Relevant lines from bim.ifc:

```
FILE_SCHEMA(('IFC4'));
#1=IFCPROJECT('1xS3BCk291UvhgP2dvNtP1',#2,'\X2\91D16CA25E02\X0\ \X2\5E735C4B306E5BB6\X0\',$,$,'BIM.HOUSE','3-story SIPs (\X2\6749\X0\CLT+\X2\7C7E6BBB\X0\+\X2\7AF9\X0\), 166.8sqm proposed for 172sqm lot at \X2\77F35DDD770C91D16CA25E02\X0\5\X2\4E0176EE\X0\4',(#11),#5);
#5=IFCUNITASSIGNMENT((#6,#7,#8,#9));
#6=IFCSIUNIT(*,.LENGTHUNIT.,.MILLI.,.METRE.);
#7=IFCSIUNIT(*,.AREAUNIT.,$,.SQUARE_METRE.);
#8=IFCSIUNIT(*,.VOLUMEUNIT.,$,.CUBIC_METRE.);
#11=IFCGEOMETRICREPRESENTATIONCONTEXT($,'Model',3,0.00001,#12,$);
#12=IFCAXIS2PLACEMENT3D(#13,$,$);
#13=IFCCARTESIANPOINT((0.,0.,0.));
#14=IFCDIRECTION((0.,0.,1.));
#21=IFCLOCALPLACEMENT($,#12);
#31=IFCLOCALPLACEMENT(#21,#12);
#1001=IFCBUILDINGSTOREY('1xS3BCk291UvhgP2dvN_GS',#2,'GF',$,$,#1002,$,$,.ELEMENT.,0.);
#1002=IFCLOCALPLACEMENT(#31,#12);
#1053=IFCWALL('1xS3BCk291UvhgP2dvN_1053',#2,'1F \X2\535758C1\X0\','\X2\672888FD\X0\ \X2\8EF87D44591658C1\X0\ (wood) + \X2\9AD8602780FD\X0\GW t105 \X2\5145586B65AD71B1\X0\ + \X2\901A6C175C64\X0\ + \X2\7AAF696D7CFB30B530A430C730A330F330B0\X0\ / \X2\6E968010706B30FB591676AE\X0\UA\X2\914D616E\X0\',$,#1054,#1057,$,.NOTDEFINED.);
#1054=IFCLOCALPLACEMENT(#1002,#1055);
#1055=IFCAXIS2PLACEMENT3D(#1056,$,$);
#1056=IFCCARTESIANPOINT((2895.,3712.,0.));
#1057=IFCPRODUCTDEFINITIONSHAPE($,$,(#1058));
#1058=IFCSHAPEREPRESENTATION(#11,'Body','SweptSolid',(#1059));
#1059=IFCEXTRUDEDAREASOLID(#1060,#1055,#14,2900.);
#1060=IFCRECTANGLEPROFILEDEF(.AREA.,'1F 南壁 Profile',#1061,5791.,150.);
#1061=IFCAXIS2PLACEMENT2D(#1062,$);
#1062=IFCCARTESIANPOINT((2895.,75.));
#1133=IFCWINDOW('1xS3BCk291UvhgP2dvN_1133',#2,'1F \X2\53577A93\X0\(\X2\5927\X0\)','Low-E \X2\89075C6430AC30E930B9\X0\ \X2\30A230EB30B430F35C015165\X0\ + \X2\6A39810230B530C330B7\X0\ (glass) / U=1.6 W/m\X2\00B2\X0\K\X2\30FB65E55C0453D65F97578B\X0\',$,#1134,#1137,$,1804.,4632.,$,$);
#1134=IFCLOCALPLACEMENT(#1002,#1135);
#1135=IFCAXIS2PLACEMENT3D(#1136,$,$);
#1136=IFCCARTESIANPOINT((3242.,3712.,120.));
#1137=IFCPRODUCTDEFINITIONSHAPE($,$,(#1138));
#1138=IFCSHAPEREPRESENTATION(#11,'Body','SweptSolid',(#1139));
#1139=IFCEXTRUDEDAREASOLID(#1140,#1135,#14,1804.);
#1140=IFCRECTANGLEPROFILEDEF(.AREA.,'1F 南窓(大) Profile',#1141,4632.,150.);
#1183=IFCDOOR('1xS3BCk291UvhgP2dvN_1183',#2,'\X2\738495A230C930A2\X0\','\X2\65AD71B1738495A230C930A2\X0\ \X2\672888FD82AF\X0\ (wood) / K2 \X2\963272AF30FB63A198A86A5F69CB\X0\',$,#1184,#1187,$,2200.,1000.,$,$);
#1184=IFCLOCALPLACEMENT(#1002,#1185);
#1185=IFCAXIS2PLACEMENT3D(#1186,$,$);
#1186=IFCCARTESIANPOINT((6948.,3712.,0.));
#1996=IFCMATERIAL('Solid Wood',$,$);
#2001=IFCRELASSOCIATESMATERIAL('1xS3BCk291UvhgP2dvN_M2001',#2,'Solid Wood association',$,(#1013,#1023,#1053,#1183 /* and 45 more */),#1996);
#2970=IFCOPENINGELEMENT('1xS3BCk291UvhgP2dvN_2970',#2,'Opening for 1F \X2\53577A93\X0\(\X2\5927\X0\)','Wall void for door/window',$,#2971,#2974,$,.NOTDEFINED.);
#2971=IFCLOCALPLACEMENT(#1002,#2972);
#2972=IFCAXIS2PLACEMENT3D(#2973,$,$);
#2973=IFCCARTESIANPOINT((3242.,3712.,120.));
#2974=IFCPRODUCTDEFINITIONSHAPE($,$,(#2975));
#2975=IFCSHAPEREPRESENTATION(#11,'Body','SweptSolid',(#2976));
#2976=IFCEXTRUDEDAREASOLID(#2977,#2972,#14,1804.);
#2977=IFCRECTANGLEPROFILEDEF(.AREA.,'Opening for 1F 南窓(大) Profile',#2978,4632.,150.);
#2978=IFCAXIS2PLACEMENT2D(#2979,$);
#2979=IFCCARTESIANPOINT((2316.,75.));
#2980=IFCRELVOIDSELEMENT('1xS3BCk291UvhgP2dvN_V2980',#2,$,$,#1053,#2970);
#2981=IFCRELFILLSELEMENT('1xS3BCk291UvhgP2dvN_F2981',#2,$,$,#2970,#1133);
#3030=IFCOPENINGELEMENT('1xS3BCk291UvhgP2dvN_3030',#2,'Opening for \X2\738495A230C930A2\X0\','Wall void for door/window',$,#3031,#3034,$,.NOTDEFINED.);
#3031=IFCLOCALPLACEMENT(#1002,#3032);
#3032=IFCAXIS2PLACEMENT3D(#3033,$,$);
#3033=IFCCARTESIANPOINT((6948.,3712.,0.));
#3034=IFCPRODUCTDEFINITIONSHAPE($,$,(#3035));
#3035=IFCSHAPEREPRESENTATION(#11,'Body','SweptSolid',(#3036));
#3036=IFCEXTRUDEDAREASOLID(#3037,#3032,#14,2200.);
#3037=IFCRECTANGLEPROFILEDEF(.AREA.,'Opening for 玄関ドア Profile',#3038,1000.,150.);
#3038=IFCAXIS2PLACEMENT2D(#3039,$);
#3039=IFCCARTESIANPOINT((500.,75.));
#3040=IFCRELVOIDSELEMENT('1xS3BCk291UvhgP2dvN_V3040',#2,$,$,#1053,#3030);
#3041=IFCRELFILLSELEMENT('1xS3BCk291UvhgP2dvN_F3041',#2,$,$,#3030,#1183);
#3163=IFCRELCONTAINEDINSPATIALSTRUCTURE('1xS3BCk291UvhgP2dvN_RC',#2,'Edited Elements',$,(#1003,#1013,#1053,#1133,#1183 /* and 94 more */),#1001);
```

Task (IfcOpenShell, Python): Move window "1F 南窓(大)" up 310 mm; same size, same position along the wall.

```python
import numpy as np
import ifcopenshell
import ifcopenshell.api.geometry
import ifcopenshell.util.placement
import ifcopenshell.util.unit

model = ifcopenshell.open("bim.ifc")
unit_scale = ifcopenshell.util.unit.calculate_unit_scale(model)

window = model.by_id(1133)
opening = window.FillsVoids[0].RelatingOpeningElement
dz = 0.31 / unit_scale

shift = np.array([0.0, 0.0, dz])
# The window is not placed relative to its opening, so move both.
for product in (opening, window):
    matrix = ifcopenshell.util.placement.get_local_placement(product.ObjectPlacement)
    matrix[:3, 3] += shift
    ifcopenshell.api.geometry.edit_object_placement(model, product=product, matrix=matrix, is_si=False)

print(f"moved by {dz * unit_scale:+.3f} m")

model.write("bim_rev.ifc")
```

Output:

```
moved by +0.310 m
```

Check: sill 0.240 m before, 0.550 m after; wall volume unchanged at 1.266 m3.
